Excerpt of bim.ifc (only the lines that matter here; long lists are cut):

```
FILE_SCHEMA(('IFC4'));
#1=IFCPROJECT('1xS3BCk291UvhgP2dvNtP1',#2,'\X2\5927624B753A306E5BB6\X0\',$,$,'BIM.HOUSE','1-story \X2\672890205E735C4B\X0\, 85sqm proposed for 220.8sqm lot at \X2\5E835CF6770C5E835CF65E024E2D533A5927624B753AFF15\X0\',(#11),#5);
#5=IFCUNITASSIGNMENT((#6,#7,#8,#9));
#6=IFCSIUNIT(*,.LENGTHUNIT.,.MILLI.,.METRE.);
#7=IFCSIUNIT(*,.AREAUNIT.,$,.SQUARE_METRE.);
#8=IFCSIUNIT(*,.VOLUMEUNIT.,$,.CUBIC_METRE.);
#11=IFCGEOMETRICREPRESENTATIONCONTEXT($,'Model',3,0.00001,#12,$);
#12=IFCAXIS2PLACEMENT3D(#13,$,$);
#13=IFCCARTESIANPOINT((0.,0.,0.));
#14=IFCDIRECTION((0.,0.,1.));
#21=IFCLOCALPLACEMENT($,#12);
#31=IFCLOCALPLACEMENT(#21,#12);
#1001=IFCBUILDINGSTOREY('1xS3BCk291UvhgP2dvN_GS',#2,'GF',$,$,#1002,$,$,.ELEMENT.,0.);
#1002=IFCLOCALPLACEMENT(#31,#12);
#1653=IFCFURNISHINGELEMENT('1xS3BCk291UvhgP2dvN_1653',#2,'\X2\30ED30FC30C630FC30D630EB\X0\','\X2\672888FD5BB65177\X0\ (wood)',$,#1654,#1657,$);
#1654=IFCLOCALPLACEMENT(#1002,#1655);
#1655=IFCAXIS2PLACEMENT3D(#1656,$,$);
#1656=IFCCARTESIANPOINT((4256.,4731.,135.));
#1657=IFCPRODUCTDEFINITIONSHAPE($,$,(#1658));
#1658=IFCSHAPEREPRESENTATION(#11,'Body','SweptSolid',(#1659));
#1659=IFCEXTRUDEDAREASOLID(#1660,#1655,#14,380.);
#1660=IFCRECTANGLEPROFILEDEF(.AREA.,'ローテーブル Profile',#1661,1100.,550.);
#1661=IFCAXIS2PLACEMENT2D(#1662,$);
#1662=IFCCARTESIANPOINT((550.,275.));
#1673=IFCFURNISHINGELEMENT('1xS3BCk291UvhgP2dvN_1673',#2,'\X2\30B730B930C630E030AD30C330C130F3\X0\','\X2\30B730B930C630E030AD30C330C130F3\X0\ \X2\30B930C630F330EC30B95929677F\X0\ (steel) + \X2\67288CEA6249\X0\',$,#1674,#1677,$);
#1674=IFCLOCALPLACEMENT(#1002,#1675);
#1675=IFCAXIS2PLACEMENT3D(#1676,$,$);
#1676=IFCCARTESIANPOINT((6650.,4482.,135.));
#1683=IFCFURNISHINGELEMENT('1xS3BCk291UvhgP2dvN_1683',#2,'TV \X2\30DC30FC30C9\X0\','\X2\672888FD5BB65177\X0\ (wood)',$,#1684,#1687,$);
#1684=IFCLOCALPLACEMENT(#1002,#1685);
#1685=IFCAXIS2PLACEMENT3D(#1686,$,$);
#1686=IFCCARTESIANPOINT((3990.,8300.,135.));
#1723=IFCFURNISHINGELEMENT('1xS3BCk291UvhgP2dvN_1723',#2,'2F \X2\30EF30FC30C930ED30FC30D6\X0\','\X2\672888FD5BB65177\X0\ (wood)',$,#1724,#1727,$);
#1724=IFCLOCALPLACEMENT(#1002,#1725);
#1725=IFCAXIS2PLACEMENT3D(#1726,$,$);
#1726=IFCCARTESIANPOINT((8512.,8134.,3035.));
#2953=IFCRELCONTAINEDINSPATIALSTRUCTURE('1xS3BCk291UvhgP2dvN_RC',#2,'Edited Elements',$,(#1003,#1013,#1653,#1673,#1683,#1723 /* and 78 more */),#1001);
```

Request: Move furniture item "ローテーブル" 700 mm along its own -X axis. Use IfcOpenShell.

```python
import ifcopenshell
import ifcopenshell.api.geometry
import ifcopenshell.util.placement
import ifcopenshell.util.unit

model = ifcopenshell.open("bim.ifc")
unit_scale = ifcopenshell.util.unit.calculate_unit_scale(model)

item = model.by_guid("1xS3BCk291UvhgP2dvN_1653")
matrix = ifcopenshell.util.placement.get_local_placement(item.ObjectPlacement)
matrix[:3, 3] -= matrix[:3, 0] * 0.7 / unit_scale
ifcopenshell.api.geometry.edit_object_placement(model, product=item, matrix=matrix, is_si=False)

print(ifcopenshell.util.placement.get_local_placement(item.ObjectPlacement).round(3) + 0.0)

model.write("bim_v2.ifc")
```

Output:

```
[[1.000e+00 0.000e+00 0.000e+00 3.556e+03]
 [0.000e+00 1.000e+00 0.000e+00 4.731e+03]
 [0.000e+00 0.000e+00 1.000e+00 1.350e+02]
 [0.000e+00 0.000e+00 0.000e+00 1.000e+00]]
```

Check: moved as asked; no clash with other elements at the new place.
